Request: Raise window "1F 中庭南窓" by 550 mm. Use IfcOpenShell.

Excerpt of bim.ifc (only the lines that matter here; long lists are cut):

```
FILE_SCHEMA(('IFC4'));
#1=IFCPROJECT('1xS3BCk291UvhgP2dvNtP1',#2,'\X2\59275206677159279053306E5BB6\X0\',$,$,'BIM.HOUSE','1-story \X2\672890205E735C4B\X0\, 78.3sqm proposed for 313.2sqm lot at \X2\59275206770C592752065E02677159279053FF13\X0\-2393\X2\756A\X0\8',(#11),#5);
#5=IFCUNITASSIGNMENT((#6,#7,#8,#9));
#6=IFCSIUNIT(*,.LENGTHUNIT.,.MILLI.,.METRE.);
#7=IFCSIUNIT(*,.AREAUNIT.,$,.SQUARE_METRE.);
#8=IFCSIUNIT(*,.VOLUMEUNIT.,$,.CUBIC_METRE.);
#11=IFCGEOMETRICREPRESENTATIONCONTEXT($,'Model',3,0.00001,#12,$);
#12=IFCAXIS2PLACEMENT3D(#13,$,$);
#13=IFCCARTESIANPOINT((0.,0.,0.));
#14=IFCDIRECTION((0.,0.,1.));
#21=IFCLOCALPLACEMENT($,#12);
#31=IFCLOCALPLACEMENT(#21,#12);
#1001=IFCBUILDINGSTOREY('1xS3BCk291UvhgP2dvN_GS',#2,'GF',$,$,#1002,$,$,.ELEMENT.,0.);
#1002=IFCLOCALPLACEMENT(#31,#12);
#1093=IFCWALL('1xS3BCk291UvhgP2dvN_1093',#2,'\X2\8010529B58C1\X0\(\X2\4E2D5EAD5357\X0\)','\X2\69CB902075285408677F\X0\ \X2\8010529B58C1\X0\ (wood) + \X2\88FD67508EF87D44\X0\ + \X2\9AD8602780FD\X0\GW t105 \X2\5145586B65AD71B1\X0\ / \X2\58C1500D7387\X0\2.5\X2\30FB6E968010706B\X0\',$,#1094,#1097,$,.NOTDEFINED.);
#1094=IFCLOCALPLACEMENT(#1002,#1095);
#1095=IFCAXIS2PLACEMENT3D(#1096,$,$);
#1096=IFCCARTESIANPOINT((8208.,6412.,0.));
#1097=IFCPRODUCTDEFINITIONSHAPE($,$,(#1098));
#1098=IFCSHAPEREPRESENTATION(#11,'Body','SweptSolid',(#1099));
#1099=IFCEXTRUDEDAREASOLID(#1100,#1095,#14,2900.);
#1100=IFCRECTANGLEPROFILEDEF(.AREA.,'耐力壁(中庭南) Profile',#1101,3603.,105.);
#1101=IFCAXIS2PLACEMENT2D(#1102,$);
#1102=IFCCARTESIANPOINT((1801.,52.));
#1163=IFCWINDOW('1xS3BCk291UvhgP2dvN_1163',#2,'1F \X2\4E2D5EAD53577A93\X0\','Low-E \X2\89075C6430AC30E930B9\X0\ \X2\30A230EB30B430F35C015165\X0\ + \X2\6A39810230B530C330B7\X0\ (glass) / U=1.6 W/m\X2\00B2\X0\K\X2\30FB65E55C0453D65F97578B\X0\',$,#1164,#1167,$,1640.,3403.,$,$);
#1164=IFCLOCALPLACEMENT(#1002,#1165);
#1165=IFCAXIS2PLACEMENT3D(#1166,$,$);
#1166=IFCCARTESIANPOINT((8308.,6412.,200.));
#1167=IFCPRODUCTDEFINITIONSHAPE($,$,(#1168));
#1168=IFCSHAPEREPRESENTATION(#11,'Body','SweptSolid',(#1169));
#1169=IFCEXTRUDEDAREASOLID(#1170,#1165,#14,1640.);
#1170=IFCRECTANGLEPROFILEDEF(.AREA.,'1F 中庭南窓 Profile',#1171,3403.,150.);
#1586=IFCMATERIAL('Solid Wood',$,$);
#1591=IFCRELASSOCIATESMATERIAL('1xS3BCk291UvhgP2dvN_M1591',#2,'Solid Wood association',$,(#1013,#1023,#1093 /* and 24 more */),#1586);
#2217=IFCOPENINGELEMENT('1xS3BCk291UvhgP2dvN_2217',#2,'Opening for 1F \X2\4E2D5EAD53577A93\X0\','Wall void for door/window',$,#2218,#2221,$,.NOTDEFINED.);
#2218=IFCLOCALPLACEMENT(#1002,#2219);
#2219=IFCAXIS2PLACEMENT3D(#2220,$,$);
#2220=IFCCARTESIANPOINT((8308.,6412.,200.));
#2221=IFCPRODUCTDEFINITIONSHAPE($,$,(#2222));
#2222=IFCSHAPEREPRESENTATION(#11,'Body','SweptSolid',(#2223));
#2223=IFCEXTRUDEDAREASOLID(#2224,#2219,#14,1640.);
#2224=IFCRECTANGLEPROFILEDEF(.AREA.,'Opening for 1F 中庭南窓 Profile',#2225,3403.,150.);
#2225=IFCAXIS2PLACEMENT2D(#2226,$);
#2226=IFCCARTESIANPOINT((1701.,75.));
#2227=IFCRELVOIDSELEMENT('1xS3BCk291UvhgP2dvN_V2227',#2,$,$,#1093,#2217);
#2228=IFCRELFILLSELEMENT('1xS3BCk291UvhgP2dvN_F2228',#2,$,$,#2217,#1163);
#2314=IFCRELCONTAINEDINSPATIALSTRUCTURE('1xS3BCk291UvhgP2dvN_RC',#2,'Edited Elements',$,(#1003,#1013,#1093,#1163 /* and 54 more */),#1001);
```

```python
import numpy as np
import ifcopenshell
import ifcopenshell.api.geometry
import ifcopenshell.util.placement
import ifcopenshell.util.unit

model = ifcopenshell.open("bim.ifc")
unit_scale = ifcopenshell.util.unit.calculate_unit_scale(model)

window = model.by_guid("1xS3BCk291UvhgP2dvN_1163")
opening = window.FillsVoids[0].RelatingOpeningElement
dz = 550.0

shift = np.array([0.0, 0.0, dz])
# The window is not placed relative to its opening, so move both.
for product in (opening, window):
    matrix = ifcopenshell.util.placement.get_local_placement(product.ObjectPlacement)
    matrix[:3, 3] += shift
    ifcopenshell.api.geometry.edit_object_placement(model, product=product, matrix=matrix, is_si=False)

print(f"moved by {dz * unit_scale:+.3f} m")

model.write("bim_rev.ifc")
```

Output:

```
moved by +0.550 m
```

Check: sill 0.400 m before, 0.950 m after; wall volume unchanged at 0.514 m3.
